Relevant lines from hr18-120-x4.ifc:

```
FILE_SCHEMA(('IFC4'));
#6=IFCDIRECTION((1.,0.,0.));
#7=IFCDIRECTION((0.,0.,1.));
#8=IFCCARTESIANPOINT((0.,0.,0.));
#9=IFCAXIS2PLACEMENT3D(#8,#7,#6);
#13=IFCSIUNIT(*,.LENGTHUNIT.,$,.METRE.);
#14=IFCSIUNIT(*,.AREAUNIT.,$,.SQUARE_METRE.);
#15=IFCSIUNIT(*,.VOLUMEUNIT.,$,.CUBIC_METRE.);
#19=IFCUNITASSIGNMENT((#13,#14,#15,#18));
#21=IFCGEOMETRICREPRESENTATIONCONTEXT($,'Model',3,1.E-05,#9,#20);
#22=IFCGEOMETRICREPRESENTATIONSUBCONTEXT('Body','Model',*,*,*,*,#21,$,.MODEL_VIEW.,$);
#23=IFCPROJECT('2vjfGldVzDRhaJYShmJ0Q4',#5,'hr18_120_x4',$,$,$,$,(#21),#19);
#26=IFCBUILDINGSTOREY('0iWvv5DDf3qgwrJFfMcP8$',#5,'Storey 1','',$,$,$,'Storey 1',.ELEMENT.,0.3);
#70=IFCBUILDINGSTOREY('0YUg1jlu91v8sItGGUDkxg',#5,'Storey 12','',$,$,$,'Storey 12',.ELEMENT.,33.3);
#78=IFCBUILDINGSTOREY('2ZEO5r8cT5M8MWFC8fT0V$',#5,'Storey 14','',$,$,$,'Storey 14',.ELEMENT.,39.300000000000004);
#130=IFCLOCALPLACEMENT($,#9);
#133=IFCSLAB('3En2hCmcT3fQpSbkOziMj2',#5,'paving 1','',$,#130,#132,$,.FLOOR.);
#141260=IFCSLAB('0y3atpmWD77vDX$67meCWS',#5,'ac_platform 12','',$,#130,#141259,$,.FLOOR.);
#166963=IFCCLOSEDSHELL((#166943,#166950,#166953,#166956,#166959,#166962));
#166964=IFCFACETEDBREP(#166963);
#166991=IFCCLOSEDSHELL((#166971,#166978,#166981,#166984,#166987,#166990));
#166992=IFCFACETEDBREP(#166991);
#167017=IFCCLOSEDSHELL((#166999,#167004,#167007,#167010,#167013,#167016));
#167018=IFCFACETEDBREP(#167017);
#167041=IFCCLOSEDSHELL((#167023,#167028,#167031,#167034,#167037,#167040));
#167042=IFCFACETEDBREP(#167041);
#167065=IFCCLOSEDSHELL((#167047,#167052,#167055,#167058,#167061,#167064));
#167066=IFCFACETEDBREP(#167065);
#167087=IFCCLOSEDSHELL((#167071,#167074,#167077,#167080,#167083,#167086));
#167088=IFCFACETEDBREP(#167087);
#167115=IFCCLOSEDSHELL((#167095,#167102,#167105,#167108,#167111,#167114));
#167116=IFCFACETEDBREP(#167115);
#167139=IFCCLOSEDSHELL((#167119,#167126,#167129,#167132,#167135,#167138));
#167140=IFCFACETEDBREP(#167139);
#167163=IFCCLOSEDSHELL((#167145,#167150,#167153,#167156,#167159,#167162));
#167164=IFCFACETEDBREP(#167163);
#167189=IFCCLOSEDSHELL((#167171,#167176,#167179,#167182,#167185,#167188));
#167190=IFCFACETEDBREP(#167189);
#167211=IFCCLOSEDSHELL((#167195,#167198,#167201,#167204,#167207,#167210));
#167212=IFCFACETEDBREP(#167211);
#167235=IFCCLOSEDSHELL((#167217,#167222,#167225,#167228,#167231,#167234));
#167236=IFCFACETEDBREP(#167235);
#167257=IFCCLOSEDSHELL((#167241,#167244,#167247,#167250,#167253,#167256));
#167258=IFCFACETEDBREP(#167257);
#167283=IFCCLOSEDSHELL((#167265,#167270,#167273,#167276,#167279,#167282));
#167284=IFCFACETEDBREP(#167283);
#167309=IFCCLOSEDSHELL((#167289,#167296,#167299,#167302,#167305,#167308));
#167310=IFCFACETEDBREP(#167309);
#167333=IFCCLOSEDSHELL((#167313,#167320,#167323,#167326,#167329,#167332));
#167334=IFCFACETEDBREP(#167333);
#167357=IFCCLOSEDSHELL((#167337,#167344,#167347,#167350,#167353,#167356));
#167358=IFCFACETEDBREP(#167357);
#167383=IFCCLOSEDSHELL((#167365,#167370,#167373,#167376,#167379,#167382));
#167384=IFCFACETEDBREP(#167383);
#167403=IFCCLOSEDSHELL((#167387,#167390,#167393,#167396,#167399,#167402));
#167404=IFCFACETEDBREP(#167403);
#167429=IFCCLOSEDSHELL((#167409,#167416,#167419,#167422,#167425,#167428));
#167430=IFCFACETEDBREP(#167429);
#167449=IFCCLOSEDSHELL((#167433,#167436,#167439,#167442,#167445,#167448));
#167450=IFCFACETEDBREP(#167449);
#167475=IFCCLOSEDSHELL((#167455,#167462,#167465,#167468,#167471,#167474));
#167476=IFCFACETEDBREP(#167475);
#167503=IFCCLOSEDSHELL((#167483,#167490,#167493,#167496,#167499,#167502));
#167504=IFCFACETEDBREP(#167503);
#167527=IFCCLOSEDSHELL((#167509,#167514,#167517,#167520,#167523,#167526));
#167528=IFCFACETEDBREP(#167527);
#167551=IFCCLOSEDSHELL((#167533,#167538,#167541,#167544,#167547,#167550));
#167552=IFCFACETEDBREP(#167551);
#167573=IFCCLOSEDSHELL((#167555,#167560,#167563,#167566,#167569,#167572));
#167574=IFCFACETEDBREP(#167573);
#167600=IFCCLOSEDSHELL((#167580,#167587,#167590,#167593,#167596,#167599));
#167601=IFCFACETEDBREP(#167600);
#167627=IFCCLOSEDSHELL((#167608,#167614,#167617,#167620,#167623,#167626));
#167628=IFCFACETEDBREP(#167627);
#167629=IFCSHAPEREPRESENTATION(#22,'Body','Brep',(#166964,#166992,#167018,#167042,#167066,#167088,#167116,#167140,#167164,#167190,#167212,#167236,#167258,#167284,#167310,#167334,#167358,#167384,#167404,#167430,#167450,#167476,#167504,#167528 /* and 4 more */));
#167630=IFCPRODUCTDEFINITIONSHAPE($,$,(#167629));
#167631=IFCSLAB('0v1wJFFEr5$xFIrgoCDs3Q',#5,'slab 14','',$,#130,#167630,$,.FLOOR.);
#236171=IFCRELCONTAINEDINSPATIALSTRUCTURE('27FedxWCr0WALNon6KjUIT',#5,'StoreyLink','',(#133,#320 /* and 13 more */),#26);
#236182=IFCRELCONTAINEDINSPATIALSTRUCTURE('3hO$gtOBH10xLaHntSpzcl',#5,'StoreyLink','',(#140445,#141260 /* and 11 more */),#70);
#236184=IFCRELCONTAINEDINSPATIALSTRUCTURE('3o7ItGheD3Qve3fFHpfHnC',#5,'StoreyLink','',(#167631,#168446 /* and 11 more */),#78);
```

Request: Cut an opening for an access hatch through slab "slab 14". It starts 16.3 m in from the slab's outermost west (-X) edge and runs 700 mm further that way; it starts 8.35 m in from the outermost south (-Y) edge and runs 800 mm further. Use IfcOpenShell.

```python
import numpy as np
import ifcopenshell
import ifcopenshell.api.feature
import ifcopenshell.api.geometry
import ifcopenshell.api.root
import ifcopenshell.geom
import ifcopenshell.util.placement
import ifcopenshell.util.representation
import ifcopenshell.util.shape
import ifcopenshell.util.unit

model = ifcopenshell.open("hr18-120-x4.ifc")
unit_scale = ifcopenshell.util.unit.calculate_unit_scale(model)
settings = ifcopenshell.geom.settings()


def volume(element):
    """Net volume in cubic metres, openings subtracted."""
    shape = ifcopenshell.geom.create_shape(settings, element)
    return ifcopenshell.util.shape.get_volume(shape.geometry)


slab = model.by_guid("0v1wJFFEr5$xFIrgoCDs3Q")
before = volume(slab)

# Extent in the slab's own axes, in metres. The edges named are its -X and -Y sides.
slab_shape = ifcopenshell.geom.create_shape(settings, slab)
vertices = ifcopenshell.util.shape.get_vertices(slab_shape.geometry)
x_min, y_min, bottom = vertices.min(axis=0)
top = vertices[:, 2].max()

opening = ifcopenshell.api.root.create_entity(model, ifc_class="IfcOpeningElement", name="Access hatch opening", predefined_type="OPENING")
context = ifcopenshell.util.representation.get_context(model, "Model", "Body", "MODEL_VIEW")
width, depth = 0.7, 0.8
outline = [(0.0, 0.0), (width, 0.0), (width, depth), (0.0, depth), (0.0, 0.0)]
# Overshoot both faces by 50 mm so the cut is clean.
shape = ifcopenshell.api.geometry.add_slab_representation(
    model, context=context, depth=top - bottom + 0.1, polyline=outline
)
ifcopenshell.api.geometry.assign_representation(model, product=opening, representation=shape)

matrix = ifcopenshell.util.placement.get_local_placement(slab.ObjectPlacement)
matrix[:, 3] = matrix @ np.append(np.array([x_min + 16.3, y_min + 8.35, bottom - 0.05]) / unit_scale, 1.0)
ifcopenshell.api.geometry.edit_object_placement(model, product=opening, matrix=matrix, is_si=False)
ifcopenshell.api.feature.add_feature(model, feature=opening, element=slab)

after = volume(slab)

print(f"slab volume {before:.3f} -> {after:.3f} m3")

model.write("hr18-120-x4-out.ifc")
```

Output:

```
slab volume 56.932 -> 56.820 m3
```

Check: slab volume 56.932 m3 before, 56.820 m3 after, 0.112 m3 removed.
